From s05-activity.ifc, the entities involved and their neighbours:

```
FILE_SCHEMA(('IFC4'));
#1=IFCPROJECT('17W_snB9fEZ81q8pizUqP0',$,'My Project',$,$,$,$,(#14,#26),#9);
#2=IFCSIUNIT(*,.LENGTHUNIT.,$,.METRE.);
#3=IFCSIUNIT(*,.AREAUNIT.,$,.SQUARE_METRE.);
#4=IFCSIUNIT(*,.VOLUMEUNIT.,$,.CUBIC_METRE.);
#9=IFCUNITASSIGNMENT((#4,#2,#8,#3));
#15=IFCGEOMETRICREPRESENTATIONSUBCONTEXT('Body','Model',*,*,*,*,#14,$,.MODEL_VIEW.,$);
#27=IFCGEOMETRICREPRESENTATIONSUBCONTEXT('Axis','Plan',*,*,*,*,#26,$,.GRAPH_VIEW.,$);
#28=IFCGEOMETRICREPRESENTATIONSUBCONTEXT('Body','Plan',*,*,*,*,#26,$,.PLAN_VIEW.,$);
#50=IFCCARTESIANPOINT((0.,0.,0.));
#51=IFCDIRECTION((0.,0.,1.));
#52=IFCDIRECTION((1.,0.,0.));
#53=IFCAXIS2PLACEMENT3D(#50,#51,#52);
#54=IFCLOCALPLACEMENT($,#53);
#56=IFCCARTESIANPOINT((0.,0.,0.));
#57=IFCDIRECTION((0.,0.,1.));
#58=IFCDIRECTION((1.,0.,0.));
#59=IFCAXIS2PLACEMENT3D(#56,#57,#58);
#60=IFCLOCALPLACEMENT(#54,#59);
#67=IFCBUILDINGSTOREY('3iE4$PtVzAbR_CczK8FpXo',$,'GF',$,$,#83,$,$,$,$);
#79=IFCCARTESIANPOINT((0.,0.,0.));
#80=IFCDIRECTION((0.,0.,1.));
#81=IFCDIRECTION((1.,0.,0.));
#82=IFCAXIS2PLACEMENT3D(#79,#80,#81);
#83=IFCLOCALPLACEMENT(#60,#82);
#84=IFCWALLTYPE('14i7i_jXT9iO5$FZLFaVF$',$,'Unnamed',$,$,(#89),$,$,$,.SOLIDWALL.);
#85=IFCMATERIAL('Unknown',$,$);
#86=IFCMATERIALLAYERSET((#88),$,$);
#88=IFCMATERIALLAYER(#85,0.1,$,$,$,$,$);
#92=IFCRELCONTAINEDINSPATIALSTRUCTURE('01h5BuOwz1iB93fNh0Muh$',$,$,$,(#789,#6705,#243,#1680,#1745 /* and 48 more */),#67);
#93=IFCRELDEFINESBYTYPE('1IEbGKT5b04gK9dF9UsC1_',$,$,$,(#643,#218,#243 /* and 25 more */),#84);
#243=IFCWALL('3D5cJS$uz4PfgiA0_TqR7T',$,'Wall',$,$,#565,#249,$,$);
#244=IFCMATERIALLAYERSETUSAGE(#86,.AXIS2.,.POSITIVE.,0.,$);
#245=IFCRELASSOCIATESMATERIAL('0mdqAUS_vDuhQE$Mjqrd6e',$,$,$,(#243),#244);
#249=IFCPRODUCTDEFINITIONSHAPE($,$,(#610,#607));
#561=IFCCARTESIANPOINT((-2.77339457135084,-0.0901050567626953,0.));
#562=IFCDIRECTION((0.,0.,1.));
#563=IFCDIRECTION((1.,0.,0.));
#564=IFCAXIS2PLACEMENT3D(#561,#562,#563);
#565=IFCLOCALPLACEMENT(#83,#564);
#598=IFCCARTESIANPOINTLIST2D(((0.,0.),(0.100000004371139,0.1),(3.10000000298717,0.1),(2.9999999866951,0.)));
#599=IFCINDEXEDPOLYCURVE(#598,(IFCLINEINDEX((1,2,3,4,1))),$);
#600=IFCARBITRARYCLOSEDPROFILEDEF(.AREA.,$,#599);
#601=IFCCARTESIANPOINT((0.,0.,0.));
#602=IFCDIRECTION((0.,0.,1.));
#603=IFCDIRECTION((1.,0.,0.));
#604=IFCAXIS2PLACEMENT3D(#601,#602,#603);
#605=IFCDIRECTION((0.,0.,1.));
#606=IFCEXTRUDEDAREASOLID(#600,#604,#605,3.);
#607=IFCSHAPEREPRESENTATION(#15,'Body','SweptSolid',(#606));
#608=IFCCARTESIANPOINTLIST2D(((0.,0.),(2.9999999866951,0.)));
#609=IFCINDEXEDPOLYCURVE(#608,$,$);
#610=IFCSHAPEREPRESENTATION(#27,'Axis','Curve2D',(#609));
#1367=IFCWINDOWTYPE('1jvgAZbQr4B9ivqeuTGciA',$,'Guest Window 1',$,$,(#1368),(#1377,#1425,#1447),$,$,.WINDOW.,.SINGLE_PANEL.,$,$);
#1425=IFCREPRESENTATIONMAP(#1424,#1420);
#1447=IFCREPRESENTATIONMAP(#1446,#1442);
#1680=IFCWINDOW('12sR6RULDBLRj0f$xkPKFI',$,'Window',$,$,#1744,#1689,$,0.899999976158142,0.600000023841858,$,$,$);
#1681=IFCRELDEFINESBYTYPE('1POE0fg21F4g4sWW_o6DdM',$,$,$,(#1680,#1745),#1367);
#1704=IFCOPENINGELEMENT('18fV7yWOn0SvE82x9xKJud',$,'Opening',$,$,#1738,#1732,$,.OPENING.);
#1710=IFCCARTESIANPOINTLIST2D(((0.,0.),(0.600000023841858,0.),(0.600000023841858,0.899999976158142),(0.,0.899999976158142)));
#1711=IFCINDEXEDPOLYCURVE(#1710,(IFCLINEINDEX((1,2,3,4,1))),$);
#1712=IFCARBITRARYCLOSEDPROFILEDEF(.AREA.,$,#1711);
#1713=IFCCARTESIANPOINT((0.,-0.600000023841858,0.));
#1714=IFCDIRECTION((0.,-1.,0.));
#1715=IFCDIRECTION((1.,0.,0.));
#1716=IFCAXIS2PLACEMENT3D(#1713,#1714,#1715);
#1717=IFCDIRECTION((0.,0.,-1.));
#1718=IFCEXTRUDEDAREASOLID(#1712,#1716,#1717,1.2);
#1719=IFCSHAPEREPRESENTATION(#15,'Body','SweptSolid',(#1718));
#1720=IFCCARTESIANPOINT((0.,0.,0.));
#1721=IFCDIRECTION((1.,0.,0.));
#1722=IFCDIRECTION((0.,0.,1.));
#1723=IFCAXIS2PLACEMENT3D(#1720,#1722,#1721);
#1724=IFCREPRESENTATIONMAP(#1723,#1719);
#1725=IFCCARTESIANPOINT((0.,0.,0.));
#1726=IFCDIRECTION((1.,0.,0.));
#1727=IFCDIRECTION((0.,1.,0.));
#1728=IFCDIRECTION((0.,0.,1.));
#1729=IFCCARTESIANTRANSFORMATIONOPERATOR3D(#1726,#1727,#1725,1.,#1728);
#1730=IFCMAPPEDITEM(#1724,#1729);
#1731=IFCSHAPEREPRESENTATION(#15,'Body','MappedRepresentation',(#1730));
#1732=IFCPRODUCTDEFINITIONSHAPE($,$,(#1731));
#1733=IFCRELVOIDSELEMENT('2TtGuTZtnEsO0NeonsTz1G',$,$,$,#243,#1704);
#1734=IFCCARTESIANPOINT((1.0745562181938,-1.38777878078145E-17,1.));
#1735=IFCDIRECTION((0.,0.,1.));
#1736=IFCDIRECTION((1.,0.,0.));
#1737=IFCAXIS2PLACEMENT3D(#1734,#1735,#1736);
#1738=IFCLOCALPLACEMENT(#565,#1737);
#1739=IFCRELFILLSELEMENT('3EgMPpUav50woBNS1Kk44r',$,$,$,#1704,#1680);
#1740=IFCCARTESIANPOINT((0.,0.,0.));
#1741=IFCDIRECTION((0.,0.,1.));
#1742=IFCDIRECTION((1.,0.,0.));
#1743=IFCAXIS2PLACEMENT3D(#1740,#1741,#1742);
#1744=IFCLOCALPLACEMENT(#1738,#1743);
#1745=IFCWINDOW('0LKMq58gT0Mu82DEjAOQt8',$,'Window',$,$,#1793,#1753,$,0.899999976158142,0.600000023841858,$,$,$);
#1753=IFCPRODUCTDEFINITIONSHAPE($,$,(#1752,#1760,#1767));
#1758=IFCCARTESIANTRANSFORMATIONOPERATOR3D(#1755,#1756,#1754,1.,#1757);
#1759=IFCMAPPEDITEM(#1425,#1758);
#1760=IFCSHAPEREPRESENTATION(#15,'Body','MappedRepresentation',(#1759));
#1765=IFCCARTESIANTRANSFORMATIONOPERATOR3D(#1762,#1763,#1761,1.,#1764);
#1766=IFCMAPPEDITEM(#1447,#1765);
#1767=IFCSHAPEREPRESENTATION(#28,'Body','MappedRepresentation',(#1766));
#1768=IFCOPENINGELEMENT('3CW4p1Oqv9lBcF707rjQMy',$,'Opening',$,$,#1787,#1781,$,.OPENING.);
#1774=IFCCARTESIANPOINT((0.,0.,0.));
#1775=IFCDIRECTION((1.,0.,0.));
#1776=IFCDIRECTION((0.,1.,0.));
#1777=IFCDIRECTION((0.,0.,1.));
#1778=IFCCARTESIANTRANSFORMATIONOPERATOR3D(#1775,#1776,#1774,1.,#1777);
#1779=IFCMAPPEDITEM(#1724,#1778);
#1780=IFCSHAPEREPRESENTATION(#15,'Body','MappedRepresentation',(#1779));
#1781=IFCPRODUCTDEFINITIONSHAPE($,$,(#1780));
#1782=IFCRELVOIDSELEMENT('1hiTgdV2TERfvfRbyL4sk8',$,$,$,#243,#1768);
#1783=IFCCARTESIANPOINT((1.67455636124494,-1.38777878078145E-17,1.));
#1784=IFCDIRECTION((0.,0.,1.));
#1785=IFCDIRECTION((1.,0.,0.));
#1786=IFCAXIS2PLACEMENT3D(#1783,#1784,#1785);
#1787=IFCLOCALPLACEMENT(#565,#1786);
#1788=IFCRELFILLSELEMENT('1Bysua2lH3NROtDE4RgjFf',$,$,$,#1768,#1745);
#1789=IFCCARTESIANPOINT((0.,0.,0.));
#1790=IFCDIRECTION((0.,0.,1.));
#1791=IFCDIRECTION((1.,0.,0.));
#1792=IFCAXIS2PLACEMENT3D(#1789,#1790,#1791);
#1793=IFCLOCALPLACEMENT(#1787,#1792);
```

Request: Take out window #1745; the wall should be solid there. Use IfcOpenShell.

```python
import ifcopenshell
import ifcopenshell.api.feature
import ifcopenshell.api.root
import ifcopenshell.geom
import ifcopenshell.util.shape

model = ifcopenshell.open("s05-activity.ifc")
settings = ifcopenshell.geom.settings()


def volume(element):
    """Net volume in cubic metres, openings subtracted."""
    shape = ifcopenshell.geom.create_shape(settings, element)
    return ifcopenshell.util.shape.get_volume(shape.geometry)


window = model.by_guid("0LKMq58gT0Mu82DEjAOQt8")
opening = window.FillsVoids[0].RelatingOpeningElement
wall = opening.VoidsElements[0].RelatingBuildingElement
before = volume(wall)

ifcopenshell.api.root.remove_product(model, product=window)
ifcopenshell.api.feature.remove_feature(model, feature=opening)

after = volume(wall)

print(f"wall volume {before:.3f} -> {after:.3f} m3")

model.write("s05-activity_rev.ifc")
```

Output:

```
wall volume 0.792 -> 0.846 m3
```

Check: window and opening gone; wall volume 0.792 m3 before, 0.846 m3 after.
